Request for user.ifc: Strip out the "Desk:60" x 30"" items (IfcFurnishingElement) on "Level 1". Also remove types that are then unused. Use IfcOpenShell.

First a look at what the model holds.

```python
import ifcopenshell
import ifcopenshell.util.element

model = ifcopenshell.open("user.ifc")
print(model.schema)
storey = next(s for s in model.by_type("IfcBuildingStorey") if s.Name == "Level 1")
furniture = [e for e in ifcopenshell.util.element.get_decomposition(storey) if e.is_a("IfcFurnishingElement")]
seen = {}
for e in furniture:
    element_type = ifcopenshell.util.element.get_type(e)
    name = element_type.Name if element_type not in (None, e) else None
    seen[name] = seen.get(name, 0) + 1
for name, count in sorted(seen.items(), key=str):
    print(count, "x", name)
```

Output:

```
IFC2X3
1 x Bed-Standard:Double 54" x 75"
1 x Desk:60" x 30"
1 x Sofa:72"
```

```python
import ifcopenshell
import ifcopenshell.api.root
import ifcopenshell.util.element

model = ifcopenshell.open("user.ifc")

storey = next(s for s in model.by_type("IfcBuildingStorey") if s.Name == "Level 1")
furniture = [e for e in ifcopenshell.util.element.get_decomposition(storey) if e.is_a("IfcFurnishingElement")]
targets = [e for e in furniture if (t := ifcopenshell.util.element.get_type(e)) not in (None, e) and t.Name == 'Desk:60" x 30"']
types = {ifcopenshell.util.element.get_type(e) for e in targets} - {None, *targets}

for e in targets:
    ifcopenshell.api.root.remove_product(model, product=e)
print(len(targets), "removed")

unused = [t for t in types if not ifcopenshell.util.element.get_types(t)]
for t in unused:
    ifcopenshell.api.root.remove_product(model, product=t)
print(len(unused), "unused types removed")

model.write("user_edited.ifc")
```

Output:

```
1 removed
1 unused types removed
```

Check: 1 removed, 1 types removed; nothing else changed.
